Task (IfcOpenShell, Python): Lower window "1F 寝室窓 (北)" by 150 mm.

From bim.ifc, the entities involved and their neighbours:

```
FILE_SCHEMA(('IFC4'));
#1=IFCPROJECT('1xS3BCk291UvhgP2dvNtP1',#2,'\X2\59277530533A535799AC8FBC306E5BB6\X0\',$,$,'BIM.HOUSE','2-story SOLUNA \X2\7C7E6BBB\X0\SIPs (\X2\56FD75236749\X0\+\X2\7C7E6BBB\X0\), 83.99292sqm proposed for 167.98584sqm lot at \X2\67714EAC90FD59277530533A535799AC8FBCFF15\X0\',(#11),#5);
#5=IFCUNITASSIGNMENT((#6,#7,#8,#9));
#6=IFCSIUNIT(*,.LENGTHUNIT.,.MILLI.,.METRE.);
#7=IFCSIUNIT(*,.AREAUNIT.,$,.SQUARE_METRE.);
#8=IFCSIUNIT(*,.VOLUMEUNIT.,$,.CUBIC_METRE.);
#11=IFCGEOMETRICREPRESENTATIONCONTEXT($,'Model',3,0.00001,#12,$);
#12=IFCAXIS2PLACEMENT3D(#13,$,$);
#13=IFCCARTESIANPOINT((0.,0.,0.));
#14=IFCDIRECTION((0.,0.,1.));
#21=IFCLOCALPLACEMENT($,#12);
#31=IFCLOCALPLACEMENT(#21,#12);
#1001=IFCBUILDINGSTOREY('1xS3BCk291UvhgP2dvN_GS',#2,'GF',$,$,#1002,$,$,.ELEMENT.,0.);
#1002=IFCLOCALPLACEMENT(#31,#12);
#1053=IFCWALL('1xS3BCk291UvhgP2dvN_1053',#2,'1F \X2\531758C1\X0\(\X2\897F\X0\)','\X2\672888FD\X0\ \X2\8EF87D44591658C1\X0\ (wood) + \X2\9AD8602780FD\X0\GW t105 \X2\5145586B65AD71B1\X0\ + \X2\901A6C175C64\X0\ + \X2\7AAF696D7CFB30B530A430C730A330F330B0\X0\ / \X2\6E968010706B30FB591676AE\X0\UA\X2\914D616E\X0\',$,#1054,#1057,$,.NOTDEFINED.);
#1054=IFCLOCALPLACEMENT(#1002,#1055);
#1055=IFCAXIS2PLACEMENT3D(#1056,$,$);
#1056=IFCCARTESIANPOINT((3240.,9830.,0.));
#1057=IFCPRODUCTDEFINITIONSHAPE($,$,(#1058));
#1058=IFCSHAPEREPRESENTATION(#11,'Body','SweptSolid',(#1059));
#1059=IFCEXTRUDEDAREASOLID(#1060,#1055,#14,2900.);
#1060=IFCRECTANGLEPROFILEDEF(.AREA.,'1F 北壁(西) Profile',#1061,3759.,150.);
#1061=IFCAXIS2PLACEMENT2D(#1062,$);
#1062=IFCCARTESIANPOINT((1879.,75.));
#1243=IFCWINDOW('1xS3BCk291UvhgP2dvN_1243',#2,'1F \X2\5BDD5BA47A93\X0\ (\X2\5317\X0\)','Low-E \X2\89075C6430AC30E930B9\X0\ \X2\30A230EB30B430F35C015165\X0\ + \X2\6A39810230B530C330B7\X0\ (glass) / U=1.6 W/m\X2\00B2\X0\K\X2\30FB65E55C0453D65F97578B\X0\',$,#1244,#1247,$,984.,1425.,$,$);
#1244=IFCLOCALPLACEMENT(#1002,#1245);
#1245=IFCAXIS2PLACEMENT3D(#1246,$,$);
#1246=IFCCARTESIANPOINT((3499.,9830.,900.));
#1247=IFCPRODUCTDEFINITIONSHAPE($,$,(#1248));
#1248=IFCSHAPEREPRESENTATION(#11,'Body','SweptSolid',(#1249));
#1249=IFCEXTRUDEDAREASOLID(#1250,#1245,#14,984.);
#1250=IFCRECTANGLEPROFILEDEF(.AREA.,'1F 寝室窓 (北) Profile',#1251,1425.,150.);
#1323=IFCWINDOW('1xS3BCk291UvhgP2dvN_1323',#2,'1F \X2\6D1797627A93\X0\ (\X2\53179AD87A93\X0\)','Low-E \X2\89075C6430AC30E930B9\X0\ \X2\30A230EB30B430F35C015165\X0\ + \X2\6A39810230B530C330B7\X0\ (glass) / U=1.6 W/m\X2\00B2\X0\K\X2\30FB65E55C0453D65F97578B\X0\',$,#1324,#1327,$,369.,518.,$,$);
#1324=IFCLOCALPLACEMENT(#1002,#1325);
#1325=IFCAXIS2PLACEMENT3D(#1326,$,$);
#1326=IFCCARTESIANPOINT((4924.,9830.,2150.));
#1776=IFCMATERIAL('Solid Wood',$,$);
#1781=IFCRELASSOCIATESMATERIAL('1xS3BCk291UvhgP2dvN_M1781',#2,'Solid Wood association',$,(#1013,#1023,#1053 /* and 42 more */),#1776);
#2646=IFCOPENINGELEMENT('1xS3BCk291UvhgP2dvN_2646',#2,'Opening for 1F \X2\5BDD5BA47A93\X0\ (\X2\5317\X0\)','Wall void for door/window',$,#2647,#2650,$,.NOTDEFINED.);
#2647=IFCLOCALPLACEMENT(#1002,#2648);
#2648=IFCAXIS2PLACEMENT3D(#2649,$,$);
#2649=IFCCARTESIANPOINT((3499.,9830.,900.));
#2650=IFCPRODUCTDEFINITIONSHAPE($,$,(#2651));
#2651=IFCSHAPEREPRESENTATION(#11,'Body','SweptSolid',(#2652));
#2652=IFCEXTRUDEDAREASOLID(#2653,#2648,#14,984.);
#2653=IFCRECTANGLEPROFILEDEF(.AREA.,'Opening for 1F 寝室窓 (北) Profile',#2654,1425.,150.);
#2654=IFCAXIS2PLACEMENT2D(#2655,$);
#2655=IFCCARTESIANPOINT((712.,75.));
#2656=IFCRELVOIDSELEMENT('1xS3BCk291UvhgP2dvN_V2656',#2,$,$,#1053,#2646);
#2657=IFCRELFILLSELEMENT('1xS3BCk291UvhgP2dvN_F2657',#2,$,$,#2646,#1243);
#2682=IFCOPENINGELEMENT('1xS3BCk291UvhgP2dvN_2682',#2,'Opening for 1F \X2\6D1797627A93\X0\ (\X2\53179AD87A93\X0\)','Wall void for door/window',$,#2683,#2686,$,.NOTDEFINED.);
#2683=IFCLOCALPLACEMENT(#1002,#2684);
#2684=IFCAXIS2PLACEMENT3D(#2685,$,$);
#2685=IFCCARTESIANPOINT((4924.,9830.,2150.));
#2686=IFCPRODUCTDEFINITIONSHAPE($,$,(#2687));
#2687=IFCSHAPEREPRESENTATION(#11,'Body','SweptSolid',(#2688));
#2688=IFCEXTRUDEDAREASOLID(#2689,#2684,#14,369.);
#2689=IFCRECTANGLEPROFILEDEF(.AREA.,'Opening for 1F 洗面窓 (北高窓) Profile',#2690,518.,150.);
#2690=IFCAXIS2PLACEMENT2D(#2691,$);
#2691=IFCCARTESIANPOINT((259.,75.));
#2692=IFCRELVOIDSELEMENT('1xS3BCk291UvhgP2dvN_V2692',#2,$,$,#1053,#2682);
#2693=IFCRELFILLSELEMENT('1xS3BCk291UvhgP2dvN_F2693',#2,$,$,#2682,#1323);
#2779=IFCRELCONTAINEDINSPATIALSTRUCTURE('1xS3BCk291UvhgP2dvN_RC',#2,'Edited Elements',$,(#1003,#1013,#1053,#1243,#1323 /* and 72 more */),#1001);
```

```python
import numpy as np
import ifcopenshell
import ifcopenshell.api.geometry
import ifcopenshell.util.placement
import ifcopenshell.util.unit

model = ifcopenshell.open("bim.ifc")
unit_scale = ifcopenshell.util.unit.calculate_unit_scale(model)

window = model.by_guid("1xS3BCk291UvhgP2dvN_1243")
opening = window.FillsVoids[0].RelatingOpeningElement
dz = -0.15 / unit_scale

shift = np.array([0.0, 0.0, dz])
# The window is not placed relative to its opening, so move both.
for product in (opening, window):
    matrix = ifcopenshell.util.placement.get_local_placement(product.ObjectPlacement)
    matrix[:3, 3] += shift
    ifcopenshell.api.geometry.edit_object_placement(model, product=product, matrix=matrix, is_si=False)

print(f"moved by {dz * unit_scale:+.3f} m")

model.write("bim-out.ifc")
```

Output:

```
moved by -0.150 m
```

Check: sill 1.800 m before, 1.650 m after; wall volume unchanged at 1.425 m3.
